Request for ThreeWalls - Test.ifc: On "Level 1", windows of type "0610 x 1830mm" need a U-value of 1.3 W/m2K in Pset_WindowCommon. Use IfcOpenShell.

First a look at what the model holds.

```python
import ifcopenshell
import ifcopenshell.util.element

model = ifcopenshell.open("ThreeWalls - Test.ifc")
print(model.schema)
storey = next(s for s in model.by_type("IfcBuildingStorey") if s.Name == "Level 1")
windows = [e for e in ifcopenshell.util.element.get_decomposition(storey) if e.is_a("IfcWindow")]
seen = {}
for e in windows:
    element_type = ifcopenshell.util.element.get_type(e)
    key = (element_type.Name if element_type != e and element_type else None, ifcopenshell.util.element.get_pset(e, "Pset_WindowCommon", "ThermalTransmittance"))
    seen[key] = seen.get(key, 0) + 1
for (name, value), count in sorted(seen.items(), key=str):
    print(count, "x", name, "|", value)
```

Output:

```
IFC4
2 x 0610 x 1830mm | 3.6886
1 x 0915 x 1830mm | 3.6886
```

```python
import ifcopenshell
import ifcopenshell.api.pset
import ifcopenshell.util.element

model = ifcopenshell.open("ThreeWalls - Test.ifc")

storey = next(s for s in model.by_type("IfcBuildingStorey") if s.Name == "Level 1")
windows = [e for e in ifcopenshell.util.element.get_decomposition(storey) if e.is_a("IfcWindow")]

count = 0
for e in windows:
    element_type = ifcopenshell.util.element.get_type(e)
    if element_type in (None, e) or element_type.Name != "0610 x 1830mm":
        continue
    # add_pset returns the element's existing set when there is one.
    pset = ifcopenshell.api.pset.add_pset(model, product=e, name="Pset_WindowCommon")
    ifcopenshell.api.pset.edit_pset(model, pset=pset, properties={"ThermalTransmittance": 1.3})
    count += 1

print(count, "windows updated")

model.write("ThreeWalls - Test-out.ifc")
```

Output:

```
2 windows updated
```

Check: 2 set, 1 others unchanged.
